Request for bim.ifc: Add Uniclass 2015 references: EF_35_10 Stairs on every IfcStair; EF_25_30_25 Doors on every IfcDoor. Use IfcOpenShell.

First a look at what the model holds.

```python
import ifcopenshell

model = ifcopenshell.open("bim.ifc")
print(model.schema)
print("classifications:", [c.Name for c in model.by_type("IfcClassification")])
for ifc_class in ("IfcDoor", "IfcRoof", "IfcStair", "IfcWall", "IfcWindow"):
    print(ifc_class, len(model.by_type(ifc_class)))
```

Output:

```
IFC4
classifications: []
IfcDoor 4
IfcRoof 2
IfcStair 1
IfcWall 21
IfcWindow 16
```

```python
import ifcopenshell
import ifcopenshell.api.classification

model = ifcopenshell.open("bim.ifc")

system = ifcopenshell.api.classification.add_classification(model, classification="Uniclass 2015")

codes = {
    "IfcStair": ("EF_35_10", "Stairs"),
    "IfcDoor": ("EF_25_30_25", "Doors"),
}
for ifc_class, (code, name) in codes.items():
    products = model.by_type(ifc_class)
    ifcopenshell.api.classification.add_reference(
        model, products=products, classification=system, identification=code, name=name
    )
    print(code, len(products))

model.write("bim-out.ifc")
```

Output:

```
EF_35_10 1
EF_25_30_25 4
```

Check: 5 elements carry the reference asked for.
